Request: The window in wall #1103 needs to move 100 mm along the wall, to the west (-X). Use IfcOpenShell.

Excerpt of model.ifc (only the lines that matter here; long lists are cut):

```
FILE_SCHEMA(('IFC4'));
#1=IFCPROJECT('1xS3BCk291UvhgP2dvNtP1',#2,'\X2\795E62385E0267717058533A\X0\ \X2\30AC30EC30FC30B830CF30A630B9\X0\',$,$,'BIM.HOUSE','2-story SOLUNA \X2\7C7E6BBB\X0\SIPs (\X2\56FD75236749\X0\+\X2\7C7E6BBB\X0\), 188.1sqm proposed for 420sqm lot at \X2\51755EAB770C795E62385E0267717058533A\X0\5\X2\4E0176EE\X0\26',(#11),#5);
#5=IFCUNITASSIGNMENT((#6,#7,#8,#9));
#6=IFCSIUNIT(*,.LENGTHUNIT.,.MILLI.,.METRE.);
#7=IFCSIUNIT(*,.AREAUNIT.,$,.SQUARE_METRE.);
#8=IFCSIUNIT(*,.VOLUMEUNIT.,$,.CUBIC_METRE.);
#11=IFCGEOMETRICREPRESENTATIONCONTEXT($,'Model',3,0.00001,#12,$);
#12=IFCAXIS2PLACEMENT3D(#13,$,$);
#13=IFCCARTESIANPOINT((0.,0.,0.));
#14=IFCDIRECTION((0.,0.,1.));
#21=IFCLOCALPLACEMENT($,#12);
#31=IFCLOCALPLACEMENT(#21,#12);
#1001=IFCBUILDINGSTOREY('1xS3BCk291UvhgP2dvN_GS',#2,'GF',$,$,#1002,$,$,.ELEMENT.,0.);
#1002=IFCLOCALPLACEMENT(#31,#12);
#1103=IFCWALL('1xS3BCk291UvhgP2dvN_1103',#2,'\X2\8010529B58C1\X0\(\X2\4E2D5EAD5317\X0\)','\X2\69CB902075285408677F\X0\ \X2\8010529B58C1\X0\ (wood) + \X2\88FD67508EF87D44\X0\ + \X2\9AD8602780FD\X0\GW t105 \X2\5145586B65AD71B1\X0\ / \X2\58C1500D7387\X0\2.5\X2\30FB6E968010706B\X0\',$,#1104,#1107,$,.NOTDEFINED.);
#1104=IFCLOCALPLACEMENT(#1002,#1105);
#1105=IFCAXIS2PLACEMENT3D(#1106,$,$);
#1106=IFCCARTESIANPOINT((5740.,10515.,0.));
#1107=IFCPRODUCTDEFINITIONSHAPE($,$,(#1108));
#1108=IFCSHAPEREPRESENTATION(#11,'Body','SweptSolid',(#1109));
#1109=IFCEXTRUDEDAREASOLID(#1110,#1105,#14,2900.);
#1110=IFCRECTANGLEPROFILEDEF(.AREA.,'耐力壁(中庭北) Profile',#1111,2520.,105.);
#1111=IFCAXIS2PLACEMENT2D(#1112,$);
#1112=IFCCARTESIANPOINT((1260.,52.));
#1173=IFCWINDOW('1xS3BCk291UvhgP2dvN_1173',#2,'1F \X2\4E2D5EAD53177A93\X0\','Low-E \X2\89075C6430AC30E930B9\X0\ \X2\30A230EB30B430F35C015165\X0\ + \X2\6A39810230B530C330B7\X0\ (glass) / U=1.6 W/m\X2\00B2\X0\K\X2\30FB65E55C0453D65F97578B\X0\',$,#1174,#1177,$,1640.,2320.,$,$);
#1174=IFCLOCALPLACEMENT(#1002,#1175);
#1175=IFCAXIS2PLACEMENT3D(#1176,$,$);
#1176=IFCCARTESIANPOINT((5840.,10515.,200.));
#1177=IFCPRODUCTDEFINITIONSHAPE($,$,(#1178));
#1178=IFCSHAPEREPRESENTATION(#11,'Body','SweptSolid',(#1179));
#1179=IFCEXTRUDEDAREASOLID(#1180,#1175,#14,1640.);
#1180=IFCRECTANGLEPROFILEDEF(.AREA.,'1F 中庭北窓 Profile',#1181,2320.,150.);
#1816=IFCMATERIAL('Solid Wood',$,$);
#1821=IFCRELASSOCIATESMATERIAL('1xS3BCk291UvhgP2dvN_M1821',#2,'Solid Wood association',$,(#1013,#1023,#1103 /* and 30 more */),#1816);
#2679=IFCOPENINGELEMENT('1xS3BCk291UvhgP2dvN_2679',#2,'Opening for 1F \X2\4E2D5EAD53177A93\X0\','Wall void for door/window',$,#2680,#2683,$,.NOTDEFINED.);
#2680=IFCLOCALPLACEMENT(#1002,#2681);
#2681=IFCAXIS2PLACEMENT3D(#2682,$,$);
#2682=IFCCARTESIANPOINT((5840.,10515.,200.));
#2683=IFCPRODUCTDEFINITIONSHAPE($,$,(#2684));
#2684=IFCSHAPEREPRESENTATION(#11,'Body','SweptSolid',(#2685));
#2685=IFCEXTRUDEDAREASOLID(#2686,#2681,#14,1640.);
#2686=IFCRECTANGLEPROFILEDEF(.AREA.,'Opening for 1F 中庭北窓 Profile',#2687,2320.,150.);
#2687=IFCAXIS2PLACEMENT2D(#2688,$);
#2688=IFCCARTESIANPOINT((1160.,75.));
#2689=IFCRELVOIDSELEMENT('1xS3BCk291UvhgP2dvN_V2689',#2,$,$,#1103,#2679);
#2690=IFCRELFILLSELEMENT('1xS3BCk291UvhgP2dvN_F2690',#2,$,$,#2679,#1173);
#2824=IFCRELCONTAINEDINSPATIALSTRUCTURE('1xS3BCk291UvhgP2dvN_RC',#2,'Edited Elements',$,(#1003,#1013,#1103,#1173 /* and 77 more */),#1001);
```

```python
import ifcopenshell
import ifcopenshell.api.geometry
import ifcopenshell.util.placement
import ifcopenshell.util.unit

model = ifcopenshell.open("model.ifc")
unit_scale = ifcopenshell.util.unit.calculate_unit_scale(model)

window = model.by_guid("1xS3BCk291UvhgP2dvN_1173")
opening = window.FillsVoids[0].RelatingOpeningElement
wall = opening.VoidsElements[0].RelatingBuildingElement

wall_matrix = ifcopenshell.util.placement.get_local_placement(wall.ObjectPlacement)
shift = wall_matrix[:3, 0] * -0.1 / unit_scale
before = ifcopenshell.util.placement.get_local_placement(window.ObjectPlacement)[:3, 3].copy()

# The window is not placed relative to its opening, so move both.
for product in (opening, window):
    matrix = ifcopenshell.util.placement.get_local_placement(product.ObjectPlacement)
    matrix[:3, 3] += shift
    ifcopenshell.api.geometry.edit_object_placement(model, product=product, matrix=matrix, is_si=False)

after = ifcopenshell.util.placement.get_local_placement(window.ObjectPlacement)[:3, 3]
print("window moved by", (after - before).round(3) + 0.0)

model.write("model_rev.ifc")
```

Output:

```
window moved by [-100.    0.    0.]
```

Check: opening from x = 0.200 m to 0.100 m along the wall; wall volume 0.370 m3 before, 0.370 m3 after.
